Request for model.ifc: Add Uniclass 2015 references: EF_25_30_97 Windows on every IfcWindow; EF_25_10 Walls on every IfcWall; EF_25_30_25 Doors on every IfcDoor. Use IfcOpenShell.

First a look at what the model holds.

```python
import ifcopenshell

model = ifcopenshell.open("model.ifc")
print(model.schema)
print("classifications:", [c.Name for c in model.by_type("IfcClassification")])
for ifc_class in ("IfcDoor", "IfcRoof", "IfcStair", "IfcWall", "IfcWindow"):
    print(ifc_class, len(model.by_type(ifc_class)))
```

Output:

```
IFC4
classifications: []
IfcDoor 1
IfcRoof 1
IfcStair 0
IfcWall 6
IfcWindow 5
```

```python
import ifcopenshell
import ifcopenshell.api.classification

model = ifcopenshell.open("model.ifc")

system = ifcopenshell.api.classification.add_classification(model, classification="Uniclass 2015")

codes = {
    "IfcWindow": ("EF_25_30_97", "Windows"),
    "IfcWall": ("EF_25_10", "Walls"),
    "IfcDoor": ("EF_25_30_25", "Doors"),
}
for ifc_class, (code, name) in codes.items():
    products = model.by_type(ifc_class)
    ifcopenshell.api.classification.add_reference(
        model, products=products, classification=system, identification=code, name=name
    )
    print(code, len(products))

model.write("model_v2.ifc")
```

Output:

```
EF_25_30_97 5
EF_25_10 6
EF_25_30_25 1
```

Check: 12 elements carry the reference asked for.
